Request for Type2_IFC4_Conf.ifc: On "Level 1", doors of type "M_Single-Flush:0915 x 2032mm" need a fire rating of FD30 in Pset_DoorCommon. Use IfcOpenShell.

First a look at what the model holds.

```python
import ifcopenshell
import ifcopenshell.util.element

model = ifcopenshell.open("Type2_IFC4_Conf.ifc")
print(model.schema)
storey = next(s for s in model.by_type("IfcBuildingStorey") if s.Name == "Level 1")
doors = [e for e in ifcopenshell.util.element.get_decomposition(storey) if e.is_a("IfcDoor")]
seen = {}
for e in doors:
    element_type = ifcopenshell.util.element.get_type(e)
    key = (element_type.Name if element_type != e and element_type else None, ifcopenshell.util.element.get_pset(e, "Pset_DoorCommon", "FireRating"))
    seen[key] = seen.get(key, 0) + 1
for (name, value), count in sorted(seen.items(), key=str):
    print(count, "x", name, "|", value)
```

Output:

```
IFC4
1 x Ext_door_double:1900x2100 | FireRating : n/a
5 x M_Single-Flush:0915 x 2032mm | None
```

```python
import ifcopenshell
import ifcopenshell.api.pset
import ifcopenshell.util.element

model = ifcopenshell.open("Type2_IFC4_Conf.ifc")

storey = next(s for s in model.by_type("IfcBuildingStorey") if s.Name == "Level 1")
doors = [e for e in ifcopenshell.util.element.get_decomposition(storey) if e.is_a("IfcDoor")]

count = 0
for e in doors:
    element_type = ifcopenshell.util.element.get_type(e)
    if element_type in (None, e) or element_type.Name != "M_Single-Flush:0915 x 2032mm":
        continue
    # add_pset returns the element's existing set when there is one.
    pset = ifcopenshell.api.pset.add_pset(model, product=e, name="Pset_DoorCommon")
    ifcopenshell.api.pset.edit_pset(model, pset=pset, properties={"FireRating": "FD30"})
    count += 1

print(count, "doors updated")

model.write("Type2_IFC4_Conf-out.ifc")
```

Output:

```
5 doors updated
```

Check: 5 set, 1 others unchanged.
